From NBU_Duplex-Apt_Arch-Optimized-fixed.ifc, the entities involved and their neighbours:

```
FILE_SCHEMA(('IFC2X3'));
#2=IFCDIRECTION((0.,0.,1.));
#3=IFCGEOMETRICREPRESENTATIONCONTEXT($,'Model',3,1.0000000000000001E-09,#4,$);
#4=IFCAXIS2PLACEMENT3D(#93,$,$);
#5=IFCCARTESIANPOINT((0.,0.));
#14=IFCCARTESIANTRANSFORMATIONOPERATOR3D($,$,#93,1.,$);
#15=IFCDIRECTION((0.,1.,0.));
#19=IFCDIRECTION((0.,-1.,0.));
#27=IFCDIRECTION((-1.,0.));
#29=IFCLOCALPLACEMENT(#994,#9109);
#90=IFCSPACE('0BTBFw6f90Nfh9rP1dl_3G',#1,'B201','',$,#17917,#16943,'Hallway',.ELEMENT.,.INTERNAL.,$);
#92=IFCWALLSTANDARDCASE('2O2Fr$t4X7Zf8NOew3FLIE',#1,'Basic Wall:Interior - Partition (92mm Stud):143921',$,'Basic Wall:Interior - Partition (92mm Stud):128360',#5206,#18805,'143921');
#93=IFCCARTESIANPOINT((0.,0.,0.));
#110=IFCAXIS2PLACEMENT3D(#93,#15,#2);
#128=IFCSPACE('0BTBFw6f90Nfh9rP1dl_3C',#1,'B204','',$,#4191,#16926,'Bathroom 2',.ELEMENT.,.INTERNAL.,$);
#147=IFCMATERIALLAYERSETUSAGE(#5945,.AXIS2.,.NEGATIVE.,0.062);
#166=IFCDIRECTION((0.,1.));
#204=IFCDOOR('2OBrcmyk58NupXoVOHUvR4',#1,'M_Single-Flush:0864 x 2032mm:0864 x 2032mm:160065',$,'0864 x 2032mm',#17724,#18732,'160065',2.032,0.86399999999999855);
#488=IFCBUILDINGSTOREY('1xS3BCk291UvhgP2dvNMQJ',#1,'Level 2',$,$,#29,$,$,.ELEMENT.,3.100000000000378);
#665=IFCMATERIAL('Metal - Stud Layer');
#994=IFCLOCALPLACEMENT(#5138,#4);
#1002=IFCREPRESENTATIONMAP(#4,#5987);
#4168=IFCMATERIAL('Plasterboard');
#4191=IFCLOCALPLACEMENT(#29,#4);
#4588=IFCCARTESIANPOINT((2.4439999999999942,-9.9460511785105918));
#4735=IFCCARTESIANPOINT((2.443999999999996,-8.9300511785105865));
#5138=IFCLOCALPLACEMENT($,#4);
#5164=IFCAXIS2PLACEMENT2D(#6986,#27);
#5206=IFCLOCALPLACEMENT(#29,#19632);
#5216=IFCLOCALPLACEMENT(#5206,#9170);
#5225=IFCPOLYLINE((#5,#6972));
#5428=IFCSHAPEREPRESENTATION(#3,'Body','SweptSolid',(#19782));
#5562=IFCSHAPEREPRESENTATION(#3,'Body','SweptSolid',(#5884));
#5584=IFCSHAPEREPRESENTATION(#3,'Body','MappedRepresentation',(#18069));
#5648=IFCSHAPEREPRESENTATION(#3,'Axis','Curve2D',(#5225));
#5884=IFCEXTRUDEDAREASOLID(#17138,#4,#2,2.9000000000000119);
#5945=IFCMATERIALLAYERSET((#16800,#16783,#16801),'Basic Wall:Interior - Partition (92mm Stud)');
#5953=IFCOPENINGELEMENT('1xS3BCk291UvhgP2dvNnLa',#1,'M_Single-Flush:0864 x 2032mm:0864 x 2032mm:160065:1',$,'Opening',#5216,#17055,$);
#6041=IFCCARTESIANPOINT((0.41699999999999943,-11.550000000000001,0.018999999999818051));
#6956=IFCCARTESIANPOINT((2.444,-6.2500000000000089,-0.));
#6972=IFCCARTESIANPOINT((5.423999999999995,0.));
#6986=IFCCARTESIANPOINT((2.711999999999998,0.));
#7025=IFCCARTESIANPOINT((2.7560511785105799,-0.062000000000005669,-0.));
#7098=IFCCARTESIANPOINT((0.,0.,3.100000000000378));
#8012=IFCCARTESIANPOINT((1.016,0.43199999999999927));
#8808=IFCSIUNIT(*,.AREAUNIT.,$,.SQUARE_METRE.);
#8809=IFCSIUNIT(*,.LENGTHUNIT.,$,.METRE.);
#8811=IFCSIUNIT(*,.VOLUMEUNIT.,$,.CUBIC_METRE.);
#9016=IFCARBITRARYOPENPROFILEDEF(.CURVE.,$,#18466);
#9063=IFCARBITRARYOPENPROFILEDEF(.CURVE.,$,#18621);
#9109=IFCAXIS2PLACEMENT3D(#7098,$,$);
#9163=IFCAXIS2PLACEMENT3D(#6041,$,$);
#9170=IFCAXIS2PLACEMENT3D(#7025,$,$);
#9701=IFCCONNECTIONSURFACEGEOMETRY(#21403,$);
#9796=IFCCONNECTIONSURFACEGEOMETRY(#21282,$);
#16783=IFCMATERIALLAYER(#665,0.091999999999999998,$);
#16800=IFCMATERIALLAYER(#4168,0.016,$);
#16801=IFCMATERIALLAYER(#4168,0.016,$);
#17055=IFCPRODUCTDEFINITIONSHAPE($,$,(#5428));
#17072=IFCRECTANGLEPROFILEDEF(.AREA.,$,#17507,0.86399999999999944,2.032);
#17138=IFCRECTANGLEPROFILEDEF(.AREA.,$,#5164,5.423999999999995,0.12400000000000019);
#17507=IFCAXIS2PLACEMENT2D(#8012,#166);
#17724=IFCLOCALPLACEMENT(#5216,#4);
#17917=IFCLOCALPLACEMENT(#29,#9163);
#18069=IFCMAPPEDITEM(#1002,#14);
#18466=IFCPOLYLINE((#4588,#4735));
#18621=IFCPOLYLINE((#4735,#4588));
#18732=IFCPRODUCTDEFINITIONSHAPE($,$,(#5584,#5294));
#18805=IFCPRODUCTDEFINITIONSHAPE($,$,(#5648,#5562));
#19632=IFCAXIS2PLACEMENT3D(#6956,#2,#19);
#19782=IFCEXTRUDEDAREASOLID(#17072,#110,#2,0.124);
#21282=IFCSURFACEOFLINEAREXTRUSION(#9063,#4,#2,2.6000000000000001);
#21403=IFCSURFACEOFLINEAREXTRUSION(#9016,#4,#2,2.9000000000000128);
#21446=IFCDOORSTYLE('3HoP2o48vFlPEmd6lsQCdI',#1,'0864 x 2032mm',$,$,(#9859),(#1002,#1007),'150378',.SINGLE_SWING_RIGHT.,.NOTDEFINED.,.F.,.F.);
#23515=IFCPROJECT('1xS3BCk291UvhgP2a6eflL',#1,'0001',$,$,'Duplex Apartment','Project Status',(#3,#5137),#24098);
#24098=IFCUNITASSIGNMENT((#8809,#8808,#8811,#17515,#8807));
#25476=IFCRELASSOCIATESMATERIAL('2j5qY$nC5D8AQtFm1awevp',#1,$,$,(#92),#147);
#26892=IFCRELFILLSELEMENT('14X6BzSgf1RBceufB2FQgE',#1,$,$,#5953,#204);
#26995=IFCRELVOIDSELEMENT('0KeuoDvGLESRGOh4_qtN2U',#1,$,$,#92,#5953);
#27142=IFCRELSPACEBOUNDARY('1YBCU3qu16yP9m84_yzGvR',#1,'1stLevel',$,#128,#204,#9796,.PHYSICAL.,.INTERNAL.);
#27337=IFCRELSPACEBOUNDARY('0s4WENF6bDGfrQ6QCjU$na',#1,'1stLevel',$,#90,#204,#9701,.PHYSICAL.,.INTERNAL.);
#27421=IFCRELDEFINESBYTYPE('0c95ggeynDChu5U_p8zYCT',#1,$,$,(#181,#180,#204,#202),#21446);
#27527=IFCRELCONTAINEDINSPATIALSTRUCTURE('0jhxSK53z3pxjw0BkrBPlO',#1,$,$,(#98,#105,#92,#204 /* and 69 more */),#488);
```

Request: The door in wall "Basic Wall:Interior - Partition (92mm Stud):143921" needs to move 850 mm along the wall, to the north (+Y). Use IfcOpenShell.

```python
import numpy as np
import ifcopenshell
import ifcopenshell.api.geometry
import ifcopenshell.util.placement
import ifcopenshell.util.unit

model = ifcopenshell.open("NBU_Duplex-Apt_Arch-Optimized-fixed.ifc")
unit_scale = ifcopenshell.util.unit.calculate_unit_scale(model)

door = model.by_guid("2OBrcmyk58NupXoVOHUvR4")
opening = door.FillsVoids[0].RelatingOpeningElement
wall = opening.VoidsElements[0].RelatingBuildingElement

wall_matrix = ifcopenshell.util.placement.get_local_placement(wall.ObjectPlacement)
shift = wall_matrix[:3, 0] * -0.85 / unit_scale
before = ifcopenshell.util.placement.get_local_placement(door.ObjectPlacement)[:3, 3].copy()

# The door is placed relative to its opening, so it follows when the opening moves.
matrix = ifcopenshell.util.placement.get_local_placement(opening.ObjectPlacement)
matrix[:3, 3] += shift
ifcopenshell.api.geometry.edit_object_placement(
    model, product=opening, matrix=matrix, is_si=False, should_transform_children=True
)

# Space boundary surfaces are stored in each space's coordinates; move them too.
for rel in door.ProvidesBoundaries:
    if not rel.ConnectionGeometry:
        continue
    surface = rel.ConnectionGeometry.SurfaceOnRelatingElement
    space_matrix = ifcopenshell.util.placement.get_local_placement(rel.RelatingSpace.ObjectPlacement)
    point = np.array(surface.Position.Location.Coordinates) + space_matrix[:3, :3].T @ shift
    surface.Position = model.createIfcAxis2Placement3D(
        model.createIfcCartesianPoint(point.tolist()), surface.Position.Axis, surface.Position.RefDirection
    )

after = ifcopenshell.util.placement.get_local_placement(door.ObjectPlacement)[:3, 3]
print("door moved by", (after - before).round(3) + 0.0)

model.write("NBU_Duplex-Apt_Arch-Optimized-fixed_updated.ifc")
```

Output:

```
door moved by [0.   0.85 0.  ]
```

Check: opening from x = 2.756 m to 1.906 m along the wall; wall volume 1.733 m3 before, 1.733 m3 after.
